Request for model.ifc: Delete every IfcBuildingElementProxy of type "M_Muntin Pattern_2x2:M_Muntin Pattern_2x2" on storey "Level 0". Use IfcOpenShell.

First a look at what the model holds.

```python
import ifcopenshell
import ifcopenshell.util.element

model = ifcopenshell.open("model.ifc")
print(model.schema)
storey = next(s for s in model.by_type("IfcBuildingStorey") if s.Name == "Level 0")
proxies = [e for e in ifcopenshell.util.element.get_decomposition(storey) if e.is_a("IfcBuildingElementProxy")]
seen = {}
for e in proxies:
    element_type = ifcopenshell.util.element.get_type(e)
    name = element_type.Name if element_type not in (None, e) else None
    seen[name] = seen.get(name, 0) + 1
for name, count in sorted(seen.items(), key=str):
    print(count, "x", name)
```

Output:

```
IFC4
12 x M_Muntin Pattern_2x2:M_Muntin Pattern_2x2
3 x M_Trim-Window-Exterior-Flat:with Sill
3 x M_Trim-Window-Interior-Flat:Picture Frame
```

```python
import ifcopenshell
import ifcopenshell.api.root
import ifcopenshell.util.element

model = ifcopenshell.open("model.ifc")

storey = next(s for s in model.by_type("IfcBuildingStorey") if s.Name == "Level 0")
proxies = [e for e in ifcopenshell.util.element.get_decomposition(storey) if e.is_a("IfcBuildingElementProxy")]
targets = [e for e in proxies if (t := ifcopenshell.util.element.get_type(e)) not in (None, e) and t.Name == "M_Muntin Pattern_2x2:M_Muntin Pattern_2x2"]

for e in targets:
    ifcopenshell.api.root.remove_product(model, product=e)
print(len(targets), "removed")

model.write("model_edited.ifc")
```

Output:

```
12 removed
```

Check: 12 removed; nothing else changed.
